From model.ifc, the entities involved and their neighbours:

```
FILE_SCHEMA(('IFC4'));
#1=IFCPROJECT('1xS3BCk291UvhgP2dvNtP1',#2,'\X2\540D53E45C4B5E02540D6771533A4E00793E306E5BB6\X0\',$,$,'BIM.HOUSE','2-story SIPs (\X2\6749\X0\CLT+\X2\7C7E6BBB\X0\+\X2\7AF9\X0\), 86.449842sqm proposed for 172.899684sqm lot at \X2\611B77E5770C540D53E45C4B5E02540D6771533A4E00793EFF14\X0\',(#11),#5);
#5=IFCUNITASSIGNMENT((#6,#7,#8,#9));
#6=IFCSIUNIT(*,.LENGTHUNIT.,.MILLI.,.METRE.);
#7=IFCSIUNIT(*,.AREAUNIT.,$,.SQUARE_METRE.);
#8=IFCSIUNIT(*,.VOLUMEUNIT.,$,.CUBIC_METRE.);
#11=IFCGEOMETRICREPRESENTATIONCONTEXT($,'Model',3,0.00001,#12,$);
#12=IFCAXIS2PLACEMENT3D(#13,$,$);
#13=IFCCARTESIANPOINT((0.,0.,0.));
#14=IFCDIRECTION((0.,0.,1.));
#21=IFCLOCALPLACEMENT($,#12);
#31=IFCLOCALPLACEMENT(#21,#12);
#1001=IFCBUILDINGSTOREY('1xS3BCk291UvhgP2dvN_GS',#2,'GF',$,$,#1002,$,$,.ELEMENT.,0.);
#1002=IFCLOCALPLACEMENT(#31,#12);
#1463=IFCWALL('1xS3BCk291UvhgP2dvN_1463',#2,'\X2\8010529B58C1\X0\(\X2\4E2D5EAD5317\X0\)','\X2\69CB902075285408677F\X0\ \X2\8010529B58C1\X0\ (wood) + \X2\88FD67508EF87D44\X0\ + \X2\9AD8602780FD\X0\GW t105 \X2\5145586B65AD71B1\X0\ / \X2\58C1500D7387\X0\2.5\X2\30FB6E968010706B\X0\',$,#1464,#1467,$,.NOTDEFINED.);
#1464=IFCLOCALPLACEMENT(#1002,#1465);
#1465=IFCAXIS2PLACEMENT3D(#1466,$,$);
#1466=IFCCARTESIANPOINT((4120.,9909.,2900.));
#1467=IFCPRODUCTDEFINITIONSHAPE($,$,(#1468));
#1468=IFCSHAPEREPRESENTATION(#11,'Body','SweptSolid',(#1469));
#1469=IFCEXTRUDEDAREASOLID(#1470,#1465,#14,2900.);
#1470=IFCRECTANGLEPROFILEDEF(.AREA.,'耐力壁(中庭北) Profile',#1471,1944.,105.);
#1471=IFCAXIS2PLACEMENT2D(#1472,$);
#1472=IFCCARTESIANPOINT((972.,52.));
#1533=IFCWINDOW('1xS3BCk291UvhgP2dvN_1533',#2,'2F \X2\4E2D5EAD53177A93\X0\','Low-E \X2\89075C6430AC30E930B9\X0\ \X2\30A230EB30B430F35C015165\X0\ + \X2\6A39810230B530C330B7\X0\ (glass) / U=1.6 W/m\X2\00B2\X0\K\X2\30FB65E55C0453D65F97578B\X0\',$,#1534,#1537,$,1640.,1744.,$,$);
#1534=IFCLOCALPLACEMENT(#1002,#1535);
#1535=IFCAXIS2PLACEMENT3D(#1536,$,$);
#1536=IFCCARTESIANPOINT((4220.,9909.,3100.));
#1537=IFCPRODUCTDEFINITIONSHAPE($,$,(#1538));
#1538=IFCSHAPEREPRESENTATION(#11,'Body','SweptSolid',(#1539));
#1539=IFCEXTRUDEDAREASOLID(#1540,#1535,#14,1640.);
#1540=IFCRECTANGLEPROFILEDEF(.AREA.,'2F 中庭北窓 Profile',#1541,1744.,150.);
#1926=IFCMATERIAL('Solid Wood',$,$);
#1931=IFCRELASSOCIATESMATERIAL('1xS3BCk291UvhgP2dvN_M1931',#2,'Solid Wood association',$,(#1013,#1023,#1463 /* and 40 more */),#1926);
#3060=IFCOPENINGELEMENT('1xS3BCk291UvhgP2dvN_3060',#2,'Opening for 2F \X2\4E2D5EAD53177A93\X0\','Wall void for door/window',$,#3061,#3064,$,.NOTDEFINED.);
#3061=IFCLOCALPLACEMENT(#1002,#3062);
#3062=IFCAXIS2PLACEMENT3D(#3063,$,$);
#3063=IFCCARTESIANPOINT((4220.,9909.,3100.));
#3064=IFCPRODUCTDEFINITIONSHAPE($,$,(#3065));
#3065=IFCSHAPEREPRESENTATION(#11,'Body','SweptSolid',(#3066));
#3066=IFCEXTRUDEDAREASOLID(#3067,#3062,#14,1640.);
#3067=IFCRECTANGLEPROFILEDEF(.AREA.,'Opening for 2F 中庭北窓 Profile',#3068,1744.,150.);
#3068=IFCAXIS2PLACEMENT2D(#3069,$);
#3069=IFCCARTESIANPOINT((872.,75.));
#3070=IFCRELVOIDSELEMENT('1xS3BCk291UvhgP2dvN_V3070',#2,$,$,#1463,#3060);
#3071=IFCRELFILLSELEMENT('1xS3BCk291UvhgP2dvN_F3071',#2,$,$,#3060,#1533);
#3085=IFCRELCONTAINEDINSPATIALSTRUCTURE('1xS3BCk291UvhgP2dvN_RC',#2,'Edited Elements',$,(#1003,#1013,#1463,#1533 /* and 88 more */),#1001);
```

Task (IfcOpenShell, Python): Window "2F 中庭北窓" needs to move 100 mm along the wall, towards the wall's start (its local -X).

```python
import ifcopenshell
import ifcopenshell.api.geometry
import ifcopenshell.util.placement
import ifcopenshell.util.unit

model = ifcopenshell.open("model.ifc")
unit_scale = ifcopenshell.util.unit.calculate_unit_scale(model)

window = model.by_guid("1xS3BCk291UvhgP2dvN_1533")
opening = window.FillsVoids[0].RelatingOpeningElement
wall = opening.VoidsElements[0].RelatingBuildingElement

wall_matrix = ifcopenshell.util.placement.get_local_placement(wall.ObjectPlacement)
shift = wall_matrix[:3, 0] * -0.1 / unit_scale
before = ifcopenshell.util.placement.get_local_placement(window.ObjectPlacement)[:3, 3].copy()

# The window is not placed relative to its opening, so move both.
for product in (opening, window):
    matrix = ifcopenshell.util.placement.get_local_placement(product.ObjectPlacement)
    matrix[:3, 3] += shift
    ifcopenshell.api.geometry.edit_object_placement(model, product=product, matrix=matrix, is_si=False)

after = ifcopenshell.util.placement.get_local_placement(window.ObjectPlacement)[:3, 3]
print("window moved by", (after - before).round(3) + 0.0)

model.write("model_updated.ifc")
```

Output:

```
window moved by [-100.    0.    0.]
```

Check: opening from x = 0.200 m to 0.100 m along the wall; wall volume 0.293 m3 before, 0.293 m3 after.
